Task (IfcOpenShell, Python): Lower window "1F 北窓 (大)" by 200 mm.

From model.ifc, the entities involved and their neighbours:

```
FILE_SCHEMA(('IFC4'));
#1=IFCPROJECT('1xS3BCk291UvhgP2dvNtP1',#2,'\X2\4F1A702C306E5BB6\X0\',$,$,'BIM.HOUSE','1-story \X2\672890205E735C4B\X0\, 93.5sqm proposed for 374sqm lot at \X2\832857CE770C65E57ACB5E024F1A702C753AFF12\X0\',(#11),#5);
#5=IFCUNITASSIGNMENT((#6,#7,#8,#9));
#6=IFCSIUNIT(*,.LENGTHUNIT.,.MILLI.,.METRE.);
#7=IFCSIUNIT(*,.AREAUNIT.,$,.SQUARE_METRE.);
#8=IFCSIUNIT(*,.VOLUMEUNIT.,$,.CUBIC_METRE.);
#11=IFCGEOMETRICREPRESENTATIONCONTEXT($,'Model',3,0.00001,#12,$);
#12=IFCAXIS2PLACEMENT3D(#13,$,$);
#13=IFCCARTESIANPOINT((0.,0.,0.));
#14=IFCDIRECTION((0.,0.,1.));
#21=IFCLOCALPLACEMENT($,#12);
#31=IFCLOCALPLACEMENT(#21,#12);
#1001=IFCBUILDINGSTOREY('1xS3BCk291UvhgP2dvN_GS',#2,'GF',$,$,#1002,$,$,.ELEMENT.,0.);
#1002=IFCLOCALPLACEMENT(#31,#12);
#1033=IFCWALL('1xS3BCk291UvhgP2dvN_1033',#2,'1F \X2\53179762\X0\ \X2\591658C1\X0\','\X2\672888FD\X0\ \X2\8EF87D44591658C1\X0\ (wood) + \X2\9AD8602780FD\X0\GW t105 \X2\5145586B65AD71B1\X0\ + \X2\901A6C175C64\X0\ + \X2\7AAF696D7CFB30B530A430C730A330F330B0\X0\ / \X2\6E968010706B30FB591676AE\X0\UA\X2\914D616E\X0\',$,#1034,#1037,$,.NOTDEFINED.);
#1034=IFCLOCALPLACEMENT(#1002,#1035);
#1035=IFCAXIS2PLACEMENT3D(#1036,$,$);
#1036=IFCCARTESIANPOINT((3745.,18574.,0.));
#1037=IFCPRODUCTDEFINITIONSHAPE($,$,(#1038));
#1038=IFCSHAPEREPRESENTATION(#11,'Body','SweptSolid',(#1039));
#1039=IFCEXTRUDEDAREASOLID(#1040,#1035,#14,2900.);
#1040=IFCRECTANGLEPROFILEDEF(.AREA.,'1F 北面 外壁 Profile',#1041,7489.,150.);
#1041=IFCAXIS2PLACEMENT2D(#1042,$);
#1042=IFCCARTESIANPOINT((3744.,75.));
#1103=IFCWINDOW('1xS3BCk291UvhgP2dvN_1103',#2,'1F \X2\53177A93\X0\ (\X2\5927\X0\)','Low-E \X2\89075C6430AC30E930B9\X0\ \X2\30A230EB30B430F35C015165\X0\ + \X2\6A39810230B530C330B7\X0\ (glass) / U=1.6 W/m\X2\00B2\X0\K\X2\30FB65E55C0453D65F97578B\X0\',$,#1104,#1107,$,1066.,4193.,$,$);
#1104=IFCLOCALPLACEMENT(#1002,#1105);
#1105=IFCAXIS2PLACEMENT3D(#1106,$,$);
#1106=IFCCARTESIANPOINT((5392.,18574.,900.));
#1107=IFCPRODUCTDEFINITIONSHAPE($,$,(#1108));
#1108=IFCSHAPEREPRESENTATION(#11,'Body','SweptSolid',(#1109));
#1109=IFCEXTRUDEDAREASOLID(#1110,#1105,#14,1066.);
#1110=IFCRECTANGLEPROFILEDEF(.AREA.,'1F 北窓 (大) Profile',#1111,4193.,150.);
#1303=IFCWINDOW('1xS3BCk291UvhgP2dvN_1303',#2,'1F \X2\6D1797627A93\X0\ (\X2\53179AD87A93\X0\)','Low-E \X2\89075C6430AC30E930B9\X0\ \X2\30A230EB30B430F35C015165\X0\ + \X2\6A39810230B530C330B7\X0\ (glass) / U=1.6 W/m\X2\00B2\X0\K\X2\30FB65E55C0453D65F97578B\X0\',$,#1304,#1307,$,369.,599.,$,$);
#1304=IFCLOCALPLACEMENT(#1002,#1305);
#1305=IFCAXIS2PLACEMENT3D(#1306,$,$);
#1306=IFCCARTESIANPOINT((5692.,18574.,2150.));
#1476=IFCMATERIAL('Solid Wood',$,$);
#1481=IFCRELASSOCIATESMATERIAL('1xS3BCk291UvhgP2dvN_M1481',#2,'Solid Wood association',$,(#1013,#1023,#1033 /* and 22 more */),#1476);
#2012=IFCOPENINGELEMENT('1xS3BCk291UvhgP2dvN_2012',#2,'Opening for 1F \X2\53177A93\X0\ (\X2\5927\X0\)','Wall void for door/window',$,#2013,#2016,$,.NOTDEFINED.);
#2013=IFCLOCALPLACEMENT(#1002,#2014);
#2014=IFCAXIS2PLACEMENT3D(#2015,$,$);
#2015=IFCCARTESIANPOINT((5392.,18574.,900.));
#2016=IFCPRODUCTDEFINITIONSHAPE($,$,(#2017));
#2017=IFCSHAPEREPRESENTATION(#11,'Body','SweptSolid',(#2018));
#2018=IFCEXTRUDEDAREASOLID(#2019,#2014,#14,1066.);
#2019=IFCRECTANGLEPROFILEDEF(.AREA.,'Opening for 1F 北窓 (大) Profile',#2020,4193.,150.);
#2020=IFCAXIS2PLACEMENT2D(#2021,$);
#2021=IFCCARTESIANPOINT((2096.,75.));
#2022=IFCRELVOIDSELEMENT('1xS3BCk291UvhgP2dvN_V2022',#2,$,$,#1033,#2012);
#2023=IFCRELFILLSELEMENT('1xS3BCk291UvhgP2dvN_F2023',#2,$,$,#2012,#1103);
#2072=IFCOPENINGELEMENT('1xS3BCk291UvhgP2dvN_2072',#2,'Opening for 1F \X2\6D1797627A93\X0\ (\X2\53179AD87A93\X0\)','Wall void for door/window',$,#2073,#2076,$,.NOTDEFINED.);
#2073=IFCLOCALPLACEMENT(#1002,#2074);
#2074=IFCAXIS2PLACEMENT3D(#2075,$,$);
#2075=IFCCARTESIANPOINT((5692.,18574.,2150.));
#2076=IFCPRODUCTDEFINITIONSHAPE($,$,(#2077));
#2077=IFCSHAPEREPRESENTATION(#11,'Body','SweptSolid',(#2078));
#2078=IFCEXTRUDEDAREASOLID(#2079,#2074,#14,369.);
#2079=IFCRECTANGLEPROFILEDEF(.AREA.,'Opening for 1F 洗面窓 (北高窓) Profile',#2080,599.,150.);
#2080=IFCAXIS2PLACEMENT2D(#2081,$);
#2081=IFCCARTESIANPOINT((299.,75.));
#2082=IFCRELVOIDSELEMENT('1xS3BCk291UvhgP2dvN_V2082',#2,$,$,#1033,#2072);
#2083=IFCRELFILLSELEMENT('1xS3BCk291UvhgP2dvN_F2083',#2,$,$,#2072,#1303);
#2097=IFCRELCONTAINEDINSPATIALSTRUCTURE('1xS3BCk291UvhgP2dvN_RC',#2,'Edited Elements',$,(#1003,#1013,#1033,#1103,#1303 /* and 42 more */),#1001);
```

```python
import numpy as np
import ifcopenshell
import ifcopenshell.api.geometry
import ifcopenshell.util.placement
import ifcopenshell.util.unit

model = ifcopenshell.open("model.ifc")
unit_scale = ifcopenshell.util.unit.calculate_unit_scale(model)

window = model.by_id(1103)
opening = window.FillsVoids[0].RelatingOpeningElement
dz = -200.0

shift = np.array([0.0, 0.0, dz])
# The window is not placed relative to its opening, so move both.
for product in (opening, window):
    matrix = ifcopenshell.util.placement.get_local_placement(product.ObjectPlacement)
    matrix[:3, 3] += shift
    ifcopenshell.api.geometry.edit_object_placement(model, product=product, matrix=matrix, is_si=False)

print(f"moved by {dz * unit_scale:+.3f} m")

model.write("model-out.ifc")
```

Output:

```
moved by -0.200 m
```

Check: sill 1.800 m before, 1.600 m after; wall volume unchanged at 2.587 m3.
